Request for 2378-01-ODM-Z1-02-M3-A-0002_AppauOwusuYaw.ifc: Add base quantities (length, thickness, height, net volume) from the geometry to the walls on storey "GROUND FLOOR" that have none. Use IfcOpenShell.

First a look at what the model holds.

```python
import ifcopenshell
import ifcopenshell.util.element
import ifcopenshell.util.unit

model = ifcopenshell.open("2378-01-ODM-Z1-02-M3-A-0002_AppauOwusuYaw.ifc")
print(model.schema)
for unit_type in ("LENGTHUNIT", "AREAUNIT", "VOLUMEUNIT"):
    print(unit_type, ifcopenshell.util.unit.calculate_unit_scale(model, unit_type))
storey = next(s for s in model.by_type("IfcBuildingStorey") if s.Name == "GROUND FLOOR")
walls = [e for e in ifcopenshell.util.element.get_decomposition(storey) if e.is_a("IfcWall")]
for e in sorted(walls, key=lambda e: e.id()):
    print(e.id(), e.is_a(), e.Name, list(ifcopenshell.util.element.get_psets(e, qtos_only=True)), sep=" | ")
```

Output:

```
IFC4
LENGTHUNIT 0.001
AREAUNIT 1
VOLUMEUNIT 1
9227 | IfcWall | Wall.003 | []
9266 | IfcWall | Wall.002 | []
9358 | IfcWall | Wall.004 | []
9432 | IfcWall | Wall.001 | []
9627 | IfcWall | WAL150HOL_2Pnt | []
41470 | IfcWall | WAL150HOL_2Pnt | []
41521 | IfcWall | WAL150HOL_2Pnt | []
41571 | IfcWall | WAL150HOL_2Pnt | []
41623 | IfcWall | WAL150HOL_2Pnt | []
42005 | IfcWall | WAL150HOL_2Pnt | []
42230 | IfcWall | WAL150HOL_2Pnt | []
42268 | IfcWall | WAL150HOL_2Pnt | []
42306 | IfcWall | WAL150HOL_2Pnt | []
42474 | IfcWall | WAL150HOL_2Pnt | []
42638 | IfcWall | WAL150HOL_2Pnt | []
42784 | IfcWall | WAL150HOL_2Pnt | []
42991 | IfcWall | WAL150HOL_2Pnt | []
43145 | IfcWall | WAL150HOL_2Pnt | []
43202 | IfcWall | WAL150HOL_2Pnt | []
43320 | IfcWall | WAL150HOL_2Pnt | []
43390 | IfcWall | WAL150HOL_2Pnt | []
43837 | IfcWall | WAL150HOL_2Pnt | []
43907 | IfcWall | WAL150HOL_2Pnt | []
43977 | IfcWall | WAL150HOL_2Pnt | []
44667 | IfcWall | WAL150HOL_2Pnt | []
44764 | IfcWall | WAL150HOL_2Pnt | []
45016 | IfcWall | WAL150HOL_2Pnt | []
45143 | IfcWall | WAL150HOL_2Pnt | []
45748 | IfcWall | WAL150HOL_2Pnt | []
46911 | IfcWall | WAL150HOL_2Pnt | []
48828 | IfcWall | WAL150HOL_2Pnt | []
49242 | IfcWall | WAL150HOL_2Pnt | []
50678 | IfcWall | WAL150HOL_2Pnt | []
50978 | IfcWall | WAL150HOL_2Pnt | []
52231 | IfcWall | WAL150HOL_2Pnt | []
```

```python
import ifcopenshell
import ifcopenshell.api.pset
import ifcopenshell.geom
import ifcopenshell.util.element
import ifcopenshell.util.shape
import ifcopenshell.util.unit

model = ifcopenshell.open("2378-01-ODM-Z1-02-M3-A-0002_AppauOwusuYaw.ifc")
unit_scale = ifcopenshell.util.unit.calculate_unit_scale(model)
volume_scale = ifcopenshell.util.unit.calculate_unit_scale(model, "VOLUMEUNIT")
settings = ifcopenshell.geom.settings()

storey = next(s for s in model.by_type("IfcBuildingStorey") if s.Name == "GROUND FLOOR")
walls = [e for e in ifcopenshell.util.element.get_decomposition(storey) if e.is_a("IfcWall")]

for e in sorted(walls, key=lambda e: e.id()):
    if ifcopenshell.util.element.get_psets(e, qtos_only=True, should_inherit=False):
        continue
    # Geometry comes back in metres, in the element's own axes.
    shape = ifcopenshell.geom.create_shape(settings, e)
    values = {
        "Length": ifcopenshell.util.shape.get_x(shape.geometry) / unit_scale,
        "Width": ifcopenshell.util.shape.get_y(shape.geometry) / unit_scale,
        "Height": ifcopenshell.util.shape.get_z(shape.geometry) / unit_scale,
        "NetVolume": ifcopenshell.util.shape.get_volume(shape.geometry) / volume_scale,
    }
    qto = ifcopenshell.api.pset.add_qto(model, product=e, name="Qto_WallBaseQuantities")
    ifcopenshell.api.pset.edit_qto(model, qto=qto, properties=values)
    print(e.id(), {k: round(v, 3) for k, v in values.items()})

model.write("2378-01-ODM-Z1-02-M3-A-0002_AppauOwusuYaw_v2.ifc")
```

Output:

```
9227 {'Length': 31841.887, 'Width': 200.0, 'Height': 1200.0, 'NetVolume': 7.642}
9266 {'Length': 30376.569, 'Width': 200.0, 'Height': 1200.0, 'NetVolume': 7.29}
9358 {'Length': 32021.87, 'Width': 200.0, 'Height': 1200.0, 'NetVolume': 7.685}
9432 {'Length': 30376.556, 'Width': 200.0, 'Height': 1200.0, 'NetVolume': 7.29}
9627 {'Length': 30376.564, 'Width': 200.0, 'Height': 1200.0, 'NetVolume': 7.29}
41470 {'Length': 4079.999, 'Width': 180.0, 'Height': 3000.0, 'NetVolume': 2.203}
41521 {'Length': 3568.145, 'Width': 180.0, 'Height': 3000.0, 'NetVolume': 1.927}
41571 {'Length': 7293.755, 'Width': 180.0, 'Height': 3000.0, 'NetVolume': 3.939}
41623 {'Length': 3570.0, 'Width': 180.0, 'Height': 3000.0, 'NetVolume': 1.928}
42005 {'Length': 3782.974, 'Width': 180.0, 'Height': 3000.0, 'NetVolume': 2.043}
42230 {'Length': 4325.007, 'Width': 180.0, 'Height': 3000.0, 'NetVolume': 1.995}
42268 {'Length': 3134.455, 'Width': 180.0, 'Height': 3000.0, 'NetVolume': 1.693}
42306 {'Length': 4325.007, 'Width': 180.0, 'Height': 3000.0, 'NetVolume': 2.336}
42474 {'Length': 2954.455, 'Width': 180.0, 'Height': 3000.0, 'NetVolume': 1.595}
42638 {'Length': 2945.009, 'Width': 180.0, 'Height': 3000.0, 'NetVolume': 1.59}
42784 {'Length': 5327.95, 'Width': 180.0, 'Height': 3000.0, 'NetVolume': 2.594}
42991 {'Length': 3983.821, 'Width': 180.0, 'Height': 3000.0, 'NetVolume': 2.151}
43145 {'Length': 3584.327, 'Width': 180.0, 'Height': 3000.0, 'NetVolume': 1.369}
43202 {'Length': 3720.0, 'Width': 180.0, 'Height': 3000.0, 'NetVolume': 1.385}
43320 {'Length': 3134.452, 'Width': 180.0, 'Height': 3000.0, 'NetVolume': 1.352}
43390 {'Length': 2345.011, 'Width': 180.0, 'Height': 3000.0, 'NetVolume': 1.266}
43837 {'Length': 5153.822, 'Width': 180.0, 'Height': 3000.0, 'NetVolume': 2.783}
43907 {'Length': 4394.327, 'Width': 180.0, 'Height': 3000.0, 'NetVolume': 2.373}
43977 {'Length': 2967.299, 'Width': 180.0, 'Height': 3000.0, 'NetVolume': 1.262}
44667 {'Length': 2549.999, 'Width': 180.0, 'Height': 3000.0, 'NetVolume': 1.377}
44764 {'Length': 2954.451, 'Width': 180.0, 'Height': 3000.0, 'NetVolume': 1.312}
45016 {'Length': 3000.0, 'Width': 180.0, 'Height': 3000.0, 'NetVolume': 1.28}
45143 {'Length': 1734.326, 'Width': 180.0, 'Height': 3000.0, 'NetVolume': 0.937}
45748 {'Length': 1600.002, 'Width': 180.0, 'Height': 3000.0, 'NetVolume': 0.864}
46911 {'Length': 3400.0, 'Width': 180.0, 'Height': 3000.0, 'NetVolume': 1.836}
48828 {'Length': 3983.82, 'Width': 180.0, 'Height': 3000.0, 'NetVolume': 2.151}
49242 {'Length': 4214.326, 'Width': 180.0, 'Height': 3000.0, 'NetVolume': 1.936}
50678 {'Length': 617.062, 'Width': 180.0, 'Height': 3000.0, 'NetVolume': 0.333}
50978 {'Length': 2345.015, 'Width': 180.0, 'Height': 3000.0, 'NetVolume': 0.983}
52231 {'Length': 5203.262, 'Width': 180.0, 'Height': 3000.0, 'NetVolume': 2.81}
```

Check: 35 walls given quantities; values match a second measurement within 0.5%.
